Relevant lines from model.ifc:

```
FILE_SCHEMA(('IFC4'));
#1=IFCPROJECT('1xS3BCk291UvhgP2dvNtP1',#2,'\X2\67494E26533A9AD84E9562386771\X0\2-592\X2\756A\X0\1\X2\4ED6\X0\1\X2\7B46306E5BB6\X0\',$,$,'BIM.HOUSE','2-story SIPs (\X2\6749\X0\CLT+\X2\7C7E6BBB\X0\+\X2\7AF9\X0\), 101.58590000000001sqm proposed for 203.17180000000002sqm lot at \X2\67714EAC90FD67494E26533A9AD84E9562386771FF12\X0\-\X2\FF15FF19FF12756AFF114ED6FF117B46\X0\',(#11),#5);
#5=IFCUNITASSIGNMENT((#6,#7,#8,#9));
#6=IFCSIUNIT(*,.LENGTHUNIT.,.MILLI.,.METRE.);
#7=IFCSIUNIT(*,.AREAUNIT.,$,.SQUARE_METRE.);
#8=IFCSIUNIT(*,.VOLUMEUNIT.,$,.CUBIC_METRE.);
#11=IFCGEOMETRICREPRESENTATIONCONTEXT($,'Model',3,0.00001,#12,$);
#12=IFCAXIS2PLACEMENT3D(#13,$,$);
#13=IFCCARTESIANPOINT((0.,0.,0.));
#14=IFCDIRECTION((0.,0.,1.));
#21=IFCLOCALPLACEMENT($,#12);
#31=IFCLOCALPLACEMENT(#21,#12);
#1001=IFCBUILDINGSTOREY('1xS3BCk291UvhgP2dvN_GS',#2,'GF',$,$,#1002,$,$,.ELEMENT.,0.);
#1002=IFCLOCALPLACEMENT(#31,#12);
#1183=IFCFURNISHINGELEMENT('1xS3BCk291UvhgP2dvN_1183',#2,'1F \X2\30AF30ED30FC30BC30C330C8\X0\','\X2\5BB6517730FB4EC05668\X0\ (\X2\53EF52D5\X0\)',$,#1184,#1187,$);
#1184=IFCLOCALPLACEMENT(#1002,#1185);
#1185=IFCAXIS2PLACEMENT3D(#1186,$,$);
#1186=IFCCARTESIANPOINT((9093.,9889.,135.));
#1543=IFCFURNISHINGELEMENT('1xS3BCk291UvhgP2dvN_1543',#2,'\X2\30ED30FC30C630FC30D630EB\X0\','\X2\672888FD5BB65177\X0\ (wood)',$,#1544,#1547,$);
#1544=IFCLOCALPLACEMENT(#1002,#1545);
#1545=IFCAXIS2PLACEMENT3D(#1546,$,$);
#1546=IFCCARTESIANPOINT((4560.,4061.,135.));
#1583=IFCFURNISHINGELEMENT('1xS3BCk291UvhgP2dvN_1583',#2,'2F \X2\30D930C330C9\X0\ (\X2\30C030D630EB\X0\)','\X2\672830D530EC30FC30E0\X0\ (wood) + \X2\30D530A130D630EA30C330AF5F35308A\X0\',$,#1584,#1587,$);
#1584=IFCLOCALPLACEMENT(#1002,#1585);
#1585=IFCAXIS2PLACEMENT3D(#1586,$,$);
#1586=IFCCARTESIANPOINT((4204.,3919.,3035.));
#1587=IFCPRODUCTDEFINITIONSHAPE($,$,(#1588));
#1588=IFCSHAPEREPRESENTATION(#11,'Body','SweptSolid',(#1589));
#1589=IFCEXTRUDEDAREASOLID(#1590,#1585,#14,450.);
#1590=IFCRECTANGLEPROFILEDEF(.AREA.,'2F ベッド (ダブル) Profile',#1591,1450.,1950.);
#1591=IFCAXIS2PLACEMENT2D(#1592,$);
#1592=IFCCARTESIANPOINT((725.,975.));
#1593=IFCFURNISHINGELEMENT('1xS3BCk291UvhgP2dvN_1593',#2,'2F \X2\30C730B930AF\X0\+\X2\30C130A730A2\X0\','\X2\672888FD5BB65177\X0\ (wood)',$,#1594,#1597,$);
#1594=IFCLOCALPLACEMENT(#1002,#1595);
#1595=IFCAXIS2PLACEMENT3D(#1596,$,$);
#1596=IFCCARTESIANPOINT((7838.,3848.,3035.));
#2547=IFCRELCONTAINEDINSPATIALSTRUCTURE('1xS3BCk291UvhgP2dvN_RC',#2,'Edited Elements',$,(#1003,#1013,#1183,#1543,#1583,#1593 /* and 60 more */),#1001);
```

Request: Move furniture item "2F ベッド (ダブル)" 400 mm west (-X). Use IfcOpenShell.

```python
import ifcopenshell
import ifcopenshell.api.geometry
import ifcopenshell.util.placement

model = ifcopenshell.open("model.ifc")

item = model.by_id(1583)
matrix = ifcopenshell.util.placement.get_local_placement(item.ObjectPlacement)
matrix[0, 3] -= 400.0
ifcopenshell.api.geometry.edit_object_placement(model, product=item, matrix=matrix, is_si=False)

print(ifcopenshell.util.placement.get_local_placement(item.ObjectPlacement).round(3) + 0.0)

model.write("model-out.ifc")
```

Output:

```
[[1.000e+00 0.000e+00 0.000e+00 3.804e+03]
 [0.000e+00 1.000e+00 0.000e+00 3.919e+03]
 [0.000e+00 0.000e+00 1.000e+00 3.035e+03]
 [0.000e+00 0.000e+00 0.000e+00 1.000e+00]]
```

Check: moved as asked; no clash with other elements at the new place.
